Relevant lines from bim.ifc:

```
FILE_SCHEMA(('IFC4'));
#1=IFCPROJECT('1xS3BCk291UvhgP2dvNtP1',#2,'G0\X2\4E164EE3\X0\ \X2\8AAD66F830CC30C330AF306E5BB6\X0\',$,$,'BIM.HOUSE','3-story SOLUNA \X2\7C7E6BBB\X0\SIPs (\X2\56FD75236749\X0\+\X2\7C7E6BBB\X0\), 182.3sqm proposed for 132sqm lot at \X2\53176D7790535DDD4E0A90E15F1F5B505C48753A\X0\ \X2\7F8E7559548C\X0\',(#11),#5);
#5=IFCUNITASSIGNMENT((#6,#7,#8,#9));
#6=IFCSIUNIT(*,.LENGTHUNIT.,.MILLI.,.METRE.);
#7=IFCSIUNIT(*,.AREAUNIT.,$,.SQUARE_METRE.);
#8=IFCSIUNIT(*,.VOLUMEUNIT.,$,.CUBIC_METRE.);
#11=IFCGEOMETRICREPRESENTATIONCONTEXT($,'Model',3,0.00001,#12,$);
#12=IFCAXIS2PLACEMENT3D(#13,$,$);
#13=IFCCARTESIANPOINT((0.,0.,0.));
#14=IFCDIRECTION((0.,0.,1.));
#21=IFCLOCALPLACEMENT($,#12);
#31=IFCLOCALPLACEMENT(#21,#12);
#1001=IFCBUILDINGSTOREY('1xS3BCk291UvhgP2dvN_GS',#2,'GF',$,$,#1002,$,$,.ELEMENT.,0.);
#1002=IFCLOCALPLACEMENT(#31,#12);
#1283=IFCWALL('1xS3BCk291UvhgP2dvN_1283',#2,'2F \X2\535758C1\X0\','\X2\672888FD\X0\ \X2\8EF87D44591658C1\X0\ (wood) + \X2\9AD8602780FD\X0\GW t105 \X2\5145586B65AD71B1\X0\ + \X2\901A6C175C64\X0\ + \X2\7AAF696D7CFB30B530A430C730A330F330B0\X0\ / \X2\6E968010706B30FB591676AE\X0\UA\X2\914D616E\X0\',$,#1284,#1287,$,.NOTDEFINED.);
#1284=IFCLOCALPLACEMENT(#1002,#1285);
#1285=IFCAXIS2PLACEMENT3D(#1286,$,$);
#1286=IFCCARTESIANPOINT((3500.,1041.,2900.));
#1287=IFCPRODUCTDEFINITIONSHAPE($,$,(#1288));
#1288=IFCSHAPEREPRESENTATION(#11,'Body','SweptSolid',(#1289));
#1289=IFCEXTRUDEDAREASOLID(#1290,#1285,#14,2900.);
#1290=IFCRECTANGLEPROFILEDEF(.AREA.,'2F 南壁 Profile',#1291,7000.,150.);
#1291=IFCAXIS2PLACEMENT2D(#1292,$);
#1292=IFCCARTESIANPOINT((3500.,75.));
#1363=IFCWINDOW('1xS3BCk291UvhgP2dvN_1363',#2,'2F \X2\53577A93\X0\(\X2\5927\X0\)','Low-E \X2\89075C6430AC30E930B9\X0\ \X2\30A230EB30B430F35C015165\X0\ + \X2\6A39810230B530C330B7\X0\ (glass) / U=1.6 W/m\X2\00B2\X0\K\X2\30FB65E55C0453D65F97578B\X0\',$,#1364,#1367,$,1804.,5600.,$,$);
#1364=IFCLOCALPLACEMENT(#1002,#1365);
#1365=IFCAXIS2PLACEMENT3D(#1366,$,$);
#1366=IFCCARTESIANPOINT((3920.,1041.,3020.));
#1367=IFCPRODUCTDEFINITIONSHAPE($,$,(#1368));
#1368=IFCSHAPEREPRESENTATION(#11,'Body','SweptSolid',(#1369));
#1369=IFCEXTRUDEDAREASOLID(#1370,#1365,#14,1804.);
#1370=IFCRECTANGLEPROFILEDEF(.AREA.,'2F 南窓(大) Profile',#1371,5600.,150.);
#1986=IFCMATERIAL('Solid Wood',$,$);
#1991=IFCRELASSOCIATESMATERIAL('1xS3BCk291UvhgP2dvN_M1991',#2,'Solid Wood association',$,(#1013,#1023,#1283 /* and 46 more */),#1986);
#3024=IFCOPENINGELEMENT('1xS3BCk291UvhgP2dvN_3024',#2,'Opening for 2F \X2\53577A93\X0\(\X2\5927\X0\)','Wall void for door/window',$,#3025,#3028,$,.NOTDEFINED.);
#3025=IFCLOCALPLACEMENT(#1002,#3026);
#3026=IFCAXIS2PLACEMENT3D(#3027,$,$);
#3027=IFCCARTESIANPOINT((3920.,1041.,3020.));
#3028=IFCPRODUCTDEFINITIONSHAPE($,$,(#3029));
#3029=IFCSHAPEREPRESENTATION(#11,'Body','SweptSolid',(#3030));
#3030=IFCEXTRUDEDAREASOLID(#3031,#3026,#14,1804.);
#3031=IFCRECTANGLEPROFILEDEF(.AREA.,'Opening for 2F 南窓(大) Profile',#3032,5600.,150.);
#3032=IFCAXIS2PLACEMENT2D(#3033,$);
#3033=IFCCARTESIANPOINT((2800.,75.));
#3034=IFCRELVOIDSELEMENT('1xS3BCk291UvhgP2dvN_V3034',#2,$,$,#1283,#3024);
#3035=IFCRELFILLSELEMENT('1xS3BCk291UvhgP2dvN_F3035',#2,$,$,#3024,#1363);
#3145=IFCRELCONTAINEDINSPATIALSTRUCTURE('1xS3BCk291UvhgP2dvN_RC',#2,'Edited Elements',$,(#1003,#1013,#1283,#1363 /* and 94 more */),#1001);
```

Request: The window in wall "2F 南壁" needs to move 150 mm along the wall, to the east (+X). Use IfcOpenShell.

```python
import ifcopenshell
import ifcopenshell.api.geometry
import ifcopenshell.util.placement
import ifcopenshell.util.unit

model = ifcopenshell.open("bim.ifc")
unit_scale = ifcopenshell.util.unit.calculate_unit_scale(model)

window = model.by_guid("1xS3BCk291UvhgP2dvN_1363")
opening = window.FillsVoids[0].RelatingOpeningElement
wall = opening.VoidsElements[0].RelatingBuildingElement

wall_matrix = ifcopenshell.util.placement.get_local_placement(wall.ObjectPlacement)
shift = wall_matrix[:3, 0] * 0.15 / unit_scale
before = ifcopenshell.util.placement.get_local_placement(window.ObjectPlacement)[:3, 3].copy()

# The window is not placed relative to its opening, so move both.
for product in (opening, window):
    matrix = ifcopenshell.util.placement.get_local_placement(product.ObjectPlacement)
    matrix[:3, 3] += shift
    ifcopenshell.api.geometry.edit_object_placement(model, product=product, matrix=matrix, is_si=False)

after = ifcopenshell.util.placement.get_local_placement(window.ObjectPlacement)[:3, 3]
print("window moved by", (after - before).round(3) + 0.0)

model.write("bim-out.ifc")
```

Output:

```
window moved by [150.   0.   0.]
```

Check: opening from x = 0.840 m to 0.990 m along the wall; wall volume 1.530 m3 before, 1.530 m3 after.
